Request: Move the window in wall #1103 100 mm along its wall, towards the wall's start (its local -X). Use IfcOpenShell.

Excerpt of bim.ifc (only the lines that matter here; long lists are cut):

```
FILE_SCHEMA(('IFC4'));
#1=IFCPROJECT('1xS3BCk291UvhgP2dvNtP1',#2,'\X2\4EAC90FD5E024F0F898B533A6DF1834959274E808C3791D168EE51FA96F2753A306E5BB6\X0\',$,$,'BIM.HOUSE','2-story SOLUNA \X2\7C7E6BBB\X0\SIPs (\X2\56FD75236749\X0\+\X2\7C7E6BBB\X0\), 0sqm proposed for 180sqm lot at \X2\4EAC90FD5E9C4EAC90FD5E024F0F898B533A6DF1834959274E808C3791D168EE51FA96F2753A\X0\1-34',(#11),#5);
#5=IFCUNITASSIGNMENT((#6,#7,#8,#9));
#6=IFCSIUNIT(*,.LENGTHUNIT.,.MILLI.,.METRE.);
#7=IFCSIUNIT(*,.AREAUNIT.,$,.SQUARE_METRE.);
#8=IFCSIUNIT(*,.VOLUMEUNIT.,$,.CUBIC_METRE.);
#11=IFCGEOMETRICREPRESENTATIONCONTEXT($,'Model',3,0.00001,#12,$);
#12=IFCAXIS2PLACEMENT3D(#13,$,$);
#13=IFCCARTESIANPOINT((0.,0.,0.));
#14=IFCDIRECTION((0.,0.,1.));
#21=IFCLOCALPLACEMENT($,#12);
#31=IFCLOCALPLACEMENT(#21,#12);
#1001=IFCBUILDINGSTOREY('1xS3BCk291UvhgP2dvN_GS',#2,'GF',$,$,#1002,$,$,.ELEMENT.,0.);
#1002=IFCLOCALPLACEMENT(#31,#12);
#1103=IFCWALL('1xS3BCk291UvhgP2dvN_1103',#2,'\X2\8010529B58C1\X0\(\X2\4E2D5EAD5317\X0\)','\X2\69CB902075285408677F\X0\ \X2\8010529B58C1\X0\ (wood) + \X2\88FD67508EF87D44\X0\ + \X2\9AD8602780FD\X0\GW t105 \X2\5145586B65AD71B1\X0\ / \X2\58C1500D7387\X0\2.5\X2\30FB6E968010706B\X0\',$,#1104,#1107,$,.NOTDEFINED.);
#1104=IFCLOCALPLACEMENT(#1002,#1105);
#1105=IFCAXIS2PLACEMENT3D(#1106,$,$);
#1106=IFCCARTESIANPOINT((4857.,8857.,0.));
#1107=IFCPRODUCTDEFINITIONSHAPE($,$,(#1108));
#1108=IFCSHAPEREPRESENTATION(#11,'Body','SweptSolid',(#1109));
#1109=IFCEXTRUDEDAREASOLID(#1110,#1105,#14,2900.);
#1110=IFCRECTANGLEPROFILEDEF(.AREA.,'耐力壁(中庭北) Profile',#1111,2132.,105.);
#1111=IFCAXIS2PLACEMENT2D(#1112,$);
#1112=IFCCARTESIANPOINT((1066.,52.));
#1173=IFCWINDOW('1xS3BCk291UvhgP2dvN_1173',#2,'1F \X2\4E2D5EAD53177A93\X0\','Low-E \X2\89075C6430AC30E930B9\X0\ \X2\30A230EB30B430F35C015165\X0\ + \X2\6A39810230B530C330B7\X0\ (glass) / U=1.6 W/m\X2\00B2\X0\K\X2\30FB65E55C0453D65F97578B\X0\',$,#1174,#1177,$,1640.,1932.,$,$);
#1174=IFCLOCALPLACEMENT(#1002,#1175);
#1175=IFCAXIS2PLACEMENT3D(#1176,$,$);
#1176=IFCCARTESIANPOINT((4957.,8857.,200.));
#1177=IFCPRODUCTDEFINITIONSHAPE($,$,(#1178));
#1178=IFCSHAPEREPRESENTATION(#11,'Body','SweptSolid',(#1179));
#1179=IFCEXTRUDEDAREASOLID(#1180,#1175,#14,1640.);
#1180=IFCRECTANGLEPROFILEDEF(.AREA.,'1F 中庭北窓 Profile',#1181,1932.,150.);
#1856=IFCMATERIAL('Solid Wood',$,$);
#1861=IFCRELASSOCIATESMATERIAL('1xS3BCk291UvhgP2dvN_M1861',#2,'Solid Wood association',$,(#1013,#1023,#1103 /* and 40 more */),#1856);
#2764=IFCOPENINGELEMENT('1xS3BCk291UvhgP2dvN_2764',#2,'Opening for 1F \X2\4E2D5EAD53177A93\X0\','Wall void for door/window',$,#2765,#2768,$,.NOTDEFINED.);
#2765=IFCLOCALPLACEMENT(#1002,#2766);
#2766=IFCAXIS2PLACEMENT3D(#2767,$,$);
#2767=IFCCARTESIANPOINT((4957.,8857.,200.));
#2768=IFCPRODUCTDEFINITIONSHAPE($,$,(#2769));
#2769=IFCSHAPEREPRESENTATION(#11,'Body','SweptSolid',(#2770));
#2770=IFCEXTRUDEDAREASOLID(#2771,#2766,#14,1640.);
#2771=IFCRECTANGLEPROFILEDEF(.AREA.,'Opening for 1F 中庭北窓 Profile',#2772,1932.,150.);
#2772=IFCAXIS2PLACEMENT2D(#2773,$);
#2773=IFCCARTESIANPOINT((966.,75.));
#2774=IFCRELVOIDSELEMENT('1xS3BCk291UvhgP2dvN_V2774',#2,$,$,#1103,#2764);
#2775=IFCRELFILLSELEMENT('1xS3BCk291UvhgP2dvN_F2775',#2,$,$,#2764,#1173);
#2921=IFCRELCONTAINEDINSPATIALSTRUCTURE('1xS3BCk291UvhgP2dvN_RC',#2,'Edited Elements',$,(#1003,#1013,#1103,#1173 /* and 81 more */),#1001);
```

```python
import ifcopenshell
import ifcopenshell.api.geometry
import ifcopenshell.util.placement

model = ifcopenshell.open("bim.ifc")

window = model.by_id(1173)
opening = window.FillsVoids[0].RelatingOpeningElement
wall = opening.VoidsElements[0].RelatingBuildingElement

wall_matrix = ifcopenshell.util.placement.get_local_placement(wall.ObjectPlacement)
shift = wall_matrix[:3, 0] * -100.0
before = ifcopenshell.util.placement.get_local_placement(window.ObjectPlacement)[:3, 3].copy()

# The window is not placed relative to its opening, so move both.
for product in (opening, window):
    matrix = ifcopenshell.util.placement.get_local_placement(product.ObjectPlacement)
    matrix[:3, 3] += shift
    ifcopenshell.api.geometry.edit_object_placement(model, product=product, matrix=matrix, is_si=False)

after = ifcopenshell.util.placement.get_local_placement(window.ObjectPlacement)[:3, 3]
print("window moved by", (after - before).round(3) + 0.0)

model.write("bim_rev.ifc")
```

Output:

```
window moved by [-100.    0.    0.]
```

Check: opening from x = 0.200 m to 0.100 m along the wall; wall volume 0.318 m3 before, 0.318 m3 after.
